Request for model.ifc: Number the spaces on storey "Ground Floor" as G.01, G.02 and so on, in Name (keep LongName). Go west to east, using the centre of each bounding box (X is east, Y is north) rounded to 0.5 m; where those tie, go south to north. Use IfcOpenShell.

First a look at what the model holds.

```python
import ifcopenshell
import ifcopenshell.util.element
import ifcopenshell.util.placement

model = ifcopenshell.open("model.ifc")
print(model.schema)
storey = next(s for s in model.by_type("IfcBuildingStorey") if s.Name == "Ground Floor")
spaces = [e for e in ifcopenshell.util.element.get_decomposition(storey) if e.is_a("IfcSpace")]
for e in sorted(spaces, key=lambda e: e.id()):
    origin = ifcopenshell.util.placement.get_local_placement(e.ObjectPlacement)[:3, 3]
    print(e.id(), e.Name, e.LongName, origin.round(2) + 0.0, sep=" | ")
```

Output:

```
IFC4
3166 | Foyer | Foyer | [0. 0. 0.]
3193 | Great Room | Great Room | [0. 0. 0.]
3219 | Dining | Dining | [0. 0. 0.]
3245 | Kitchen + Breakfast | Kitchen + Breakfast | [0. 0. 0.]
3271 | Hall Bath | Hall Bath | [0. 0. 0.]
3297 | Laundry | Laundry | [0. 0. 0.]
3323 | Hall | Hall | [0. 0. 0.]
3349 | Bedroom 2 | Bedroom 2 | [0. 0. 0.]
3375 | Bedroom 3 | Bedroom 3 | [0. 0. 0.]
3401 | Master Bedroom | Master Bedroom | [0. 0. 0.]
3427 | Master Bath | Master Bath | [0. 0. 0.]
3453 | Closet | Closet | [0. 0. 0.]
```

```python
import ifcopenshell
import ifcopenshell.geom
import ifcopenshell.util.element
import ifcopenshell.util.shape

model = ifcopenshell.open("model.ifc")
settings = ifcopenshell.geom.settings()
settings.set("use-world-coords", True)


def centre(element):
    shape = ifcopenshell.geom.create_shape(settings, element)
    return ifcopenshell.util.shape.get_bbox_centroid(shape.geometry)


storey = next(s for s in model.by_type("IfcBuildingStorey") if s.Name == "Ground Floor")
spaces = [e for e in ifcopenshell.util.element.get_decomposition(storey) if e.is_a("IfcSpace")]

# Insertion points can sit at a corner or the storey origin, so sort by the geometry (in metres).
centres = {e: centre(e) for e in spaces}
spaces.sort(key=lambda e: (round(centres[e][0] / 0.5), centres[e][1]))

for i, e in enumerate(spaces, start=1):
    number = f"G.{i:02d}"
    e.Name = number
    print(e.id(), number)

model.write("model_edited.ifc")
```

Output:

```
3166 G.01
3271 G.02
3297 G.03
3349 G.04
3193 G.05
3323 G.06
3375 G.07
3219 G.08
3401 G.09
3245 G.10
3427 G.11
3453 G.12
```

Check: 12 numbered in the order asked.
